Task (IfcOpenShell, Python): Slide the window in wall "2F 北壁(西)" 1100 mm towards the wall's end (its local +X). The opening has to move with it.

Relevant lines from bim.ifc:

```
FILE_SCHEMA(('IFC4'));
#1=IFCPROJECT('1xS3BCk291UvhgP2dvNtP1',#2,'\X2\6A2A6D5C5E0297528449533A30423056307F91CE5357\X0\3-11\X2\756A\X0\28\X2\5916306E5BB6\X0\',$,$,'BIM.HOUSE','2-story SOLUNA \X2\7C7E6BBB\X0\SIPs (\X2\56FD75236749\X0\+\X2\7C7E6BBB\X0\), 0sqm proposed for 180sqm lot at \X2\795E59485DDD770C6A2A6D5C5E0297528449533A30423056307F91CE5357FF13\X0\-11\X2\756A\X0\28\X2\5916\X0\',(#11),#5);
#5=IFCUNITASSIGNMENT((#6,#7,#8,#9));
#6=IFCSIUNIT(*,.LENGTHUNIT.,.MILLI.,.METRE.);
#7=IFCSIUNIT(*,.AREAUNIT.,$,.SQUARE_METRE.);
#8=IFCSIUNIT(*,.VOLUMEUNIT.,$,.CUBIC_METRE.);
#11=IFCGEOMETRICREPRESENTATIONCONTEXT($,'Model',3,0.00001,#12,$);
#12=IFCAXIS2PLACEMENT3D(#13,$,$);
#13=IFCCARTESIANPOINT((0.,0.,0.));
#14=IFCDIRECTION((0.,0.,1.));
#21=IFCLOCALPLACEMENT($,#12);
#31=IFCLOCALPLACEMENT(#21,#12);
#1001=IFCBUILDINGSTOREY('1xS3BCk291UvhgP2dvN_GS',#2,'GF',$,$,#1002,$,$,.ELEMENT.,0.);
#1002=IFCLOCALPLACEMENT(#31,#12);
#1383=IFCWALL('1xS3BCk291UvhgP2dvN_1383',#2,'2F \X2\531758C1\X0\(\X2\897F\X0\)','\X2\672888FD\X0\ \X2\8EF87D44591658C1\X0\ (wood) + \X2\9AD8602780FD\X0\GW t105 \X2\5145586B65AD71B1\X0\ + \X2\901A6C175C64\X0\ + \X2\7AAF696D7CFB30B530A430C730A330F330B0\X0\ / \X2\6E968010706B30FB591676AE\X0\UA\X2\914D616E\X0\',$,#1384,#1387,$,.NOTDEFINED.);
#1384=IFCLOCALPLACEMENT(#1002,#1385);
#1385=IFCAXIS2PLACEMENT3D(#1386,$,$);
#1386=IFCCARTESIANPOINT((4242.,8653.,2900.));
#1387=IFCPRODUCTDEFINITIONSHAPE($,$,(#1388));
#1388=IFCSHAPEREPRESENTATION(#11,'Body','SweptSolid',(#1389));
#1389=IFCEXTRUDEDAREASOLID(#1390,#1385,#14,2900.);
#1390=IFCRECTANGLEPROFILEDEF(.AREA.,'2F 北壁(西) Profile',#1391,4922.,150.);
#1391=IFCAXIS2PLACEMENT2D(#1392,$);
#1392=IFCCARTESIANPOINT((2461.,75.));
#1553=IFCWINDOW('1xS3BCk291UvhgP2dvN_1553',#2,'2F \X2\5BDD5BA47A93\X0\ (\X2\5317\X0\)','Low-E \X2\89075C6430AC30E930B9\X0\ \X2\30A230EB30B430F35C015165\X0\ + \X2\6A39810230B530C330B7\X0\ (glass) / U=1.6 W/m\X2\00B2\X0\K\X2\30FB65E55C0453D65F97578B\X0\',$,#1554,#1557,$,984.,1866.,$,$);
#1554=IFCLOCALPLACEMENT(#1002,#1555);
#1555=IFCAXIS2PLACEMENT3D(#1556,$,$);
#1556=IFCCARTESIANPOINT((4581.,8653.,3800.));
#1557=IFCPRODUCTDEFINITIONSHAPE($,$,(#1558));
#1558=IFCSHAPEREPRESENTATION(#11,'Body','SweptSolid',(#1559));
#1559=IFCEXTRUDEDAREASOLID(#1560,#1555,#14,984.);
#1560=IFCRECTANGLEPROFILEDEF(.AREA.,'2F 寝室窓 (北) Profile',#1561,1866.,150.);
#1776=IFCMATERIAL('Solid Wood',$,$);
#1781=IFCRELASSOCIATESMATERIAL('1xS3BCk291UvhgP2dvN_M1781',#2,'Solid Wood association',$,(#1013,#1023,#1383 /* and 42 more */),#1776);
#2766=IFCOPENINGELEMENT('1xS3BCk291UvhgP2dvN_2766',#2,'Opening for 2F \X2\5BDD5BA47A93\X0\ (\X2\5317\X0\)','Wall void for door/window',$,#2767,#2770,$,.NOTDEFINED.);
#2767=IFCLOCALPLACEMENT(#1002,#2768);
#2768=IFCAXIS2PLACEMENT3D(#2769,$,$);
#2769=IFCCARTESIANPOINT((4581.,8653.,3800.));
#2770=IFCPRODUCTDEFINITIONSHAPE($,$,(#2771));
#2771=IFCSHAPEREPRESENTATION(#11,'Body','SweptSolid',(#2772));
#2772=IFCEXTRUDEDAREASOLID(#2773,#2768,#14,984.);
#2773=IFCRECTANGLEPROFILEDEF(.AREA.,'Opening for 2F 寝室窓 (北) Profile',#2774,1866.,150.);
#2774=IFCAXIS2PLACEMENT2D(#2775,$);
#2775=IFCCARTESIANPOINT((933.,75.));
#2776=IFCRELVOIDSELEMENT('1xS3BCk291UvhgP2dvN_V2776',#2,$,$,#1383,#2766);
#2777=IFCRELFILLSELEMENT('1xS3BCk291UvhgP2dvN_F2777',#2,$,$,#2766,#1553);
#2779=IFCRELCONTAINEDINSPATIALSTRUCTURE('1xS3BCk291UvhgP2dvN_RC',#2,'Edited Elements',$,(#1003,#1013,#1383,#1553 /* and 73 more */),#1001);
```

```python
import ifcopenshell
import ifcopenshell.api.geometry
import ifcopenshell.util.placement
import ifcopenshell.util.unit

model = ifcopenshell.open("bim.ifc")
unit_scale = ifcopenshell.util.unit.calculate_unit_scale(model)

window = model.by_guid("1xS3BCk291UvhgP2dvN_1553")
opening = window.FillsVoids[0].RelatingOpeningElement
wall = opening.VoidsElements[0].RelatingBuildingElement

wall_matrix = ifcopenshell.util.placement.get_local_placement(wall.ObjectPlacement)
shift = wall_matrix[:3, 0] * 1.1 / unit_scale
before = ifcopenshell.util.placement.get_local_placement(window.ObjectPlacement)[:3, 3].copy()

# The window is not placed relative to its opening, so move both.
for product in (opening, window):
    matrix = ifcopenshell.util.placement.get_local_placement(product.ObjectPlacement)
    matrix[:3, 3] += shift
    ifcopenshell.api.geometry.edit_object_placement(model, product=product, matrix=matrix, is_si=False)

after = ifcopenshell.util.placement.get_local_placement(window.ObjectPlacement)[:3, 3]
print("window moved by", (after - before).round(3) + 0.0)

model.write("bim_edited.ifc")
```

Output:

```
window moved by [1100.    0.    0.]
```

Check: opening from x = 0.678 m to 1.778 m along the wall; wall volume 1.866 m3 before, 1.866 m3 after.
